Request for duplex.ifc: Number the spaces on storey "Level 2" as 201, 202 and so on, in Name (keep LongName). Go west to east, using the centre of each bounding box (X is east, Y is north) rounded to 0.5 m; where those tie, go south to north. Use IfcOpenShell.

First a look at what the model holds.

```python
import ifcopenshell
import ifcopenshell.util.element
import ifcopenshell.util.placement

model = ifcopenshell.open("duplex.ifc")
print(model.schema)
storey = next(s for s in model.by_type("IfcBuildingStorey") if s.Name == "Level 2")
spaces = [e for e in ifcopenshell.util.element.get_decomposition(storey) if e.is_a("IfcSpace")]
for e in sorted(spaces, key=lambda e: e.id()):
    origin = ifcopenshell.util.placement.get_local_placement(e.ObjectPlacement)[:3, 3]
    print(e.id(), e.Name, e.LongName, origin.round(2) + 0.0, sep=" | ")
```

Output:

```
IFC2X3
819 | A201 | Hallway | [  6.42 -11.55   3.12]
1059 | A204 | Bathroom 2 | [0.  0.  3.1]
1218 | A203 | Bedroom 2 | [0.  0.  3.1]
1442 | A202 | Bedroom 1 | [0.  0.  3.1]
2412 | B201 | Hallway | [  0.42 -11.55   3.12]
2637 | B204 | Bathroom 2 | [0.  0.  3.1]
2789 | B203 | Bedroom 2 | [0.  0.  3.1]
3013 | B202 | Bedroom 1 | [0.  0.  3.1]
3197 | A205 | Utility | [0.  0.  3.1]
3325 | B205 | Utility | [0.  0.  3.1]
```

```python
import ifcopenshell
import ifcopenshell.geom
import ifcopenshell.util.element
import ifcopenshell.util.shape

model = ifcopenshell.open("duplex.ifc")
settings = ifcopenshell.geom.settings()
settings.set("use-world-coords", True)


def centre(element):
    shape = ifcopenshell.geom.create_shape(settings, element)
    return ifcopenshell.util.shape.get_bbox_centroid(shape.geometry)


storey = next(s for s in model.by_type("IfcBuildingStorey") if s.Name == "Level 2")
spaces = [e for e in ifcopenshell.util.element.get_decomposition(storey) if e.is_a("IfcSpace")]

# Insertion points can sit at a corner or the storey origin, so sort by the geometry (in metres).
centres = {e: centre(e) for e in spaces}
spaces.sort(key=lambda e: (round(centres[e][0] / 0.5), centres[e][1]))

for i, e in enumerate(spaces, start=1):
    number = f"2{i:02d}"
    e.Name = number
    print(e.id(), number)

model.write("duplex_updated.ifc")
```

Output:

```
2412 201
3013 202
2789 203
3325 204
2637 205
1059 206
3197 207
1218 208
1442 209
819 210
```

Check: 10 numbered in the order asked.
